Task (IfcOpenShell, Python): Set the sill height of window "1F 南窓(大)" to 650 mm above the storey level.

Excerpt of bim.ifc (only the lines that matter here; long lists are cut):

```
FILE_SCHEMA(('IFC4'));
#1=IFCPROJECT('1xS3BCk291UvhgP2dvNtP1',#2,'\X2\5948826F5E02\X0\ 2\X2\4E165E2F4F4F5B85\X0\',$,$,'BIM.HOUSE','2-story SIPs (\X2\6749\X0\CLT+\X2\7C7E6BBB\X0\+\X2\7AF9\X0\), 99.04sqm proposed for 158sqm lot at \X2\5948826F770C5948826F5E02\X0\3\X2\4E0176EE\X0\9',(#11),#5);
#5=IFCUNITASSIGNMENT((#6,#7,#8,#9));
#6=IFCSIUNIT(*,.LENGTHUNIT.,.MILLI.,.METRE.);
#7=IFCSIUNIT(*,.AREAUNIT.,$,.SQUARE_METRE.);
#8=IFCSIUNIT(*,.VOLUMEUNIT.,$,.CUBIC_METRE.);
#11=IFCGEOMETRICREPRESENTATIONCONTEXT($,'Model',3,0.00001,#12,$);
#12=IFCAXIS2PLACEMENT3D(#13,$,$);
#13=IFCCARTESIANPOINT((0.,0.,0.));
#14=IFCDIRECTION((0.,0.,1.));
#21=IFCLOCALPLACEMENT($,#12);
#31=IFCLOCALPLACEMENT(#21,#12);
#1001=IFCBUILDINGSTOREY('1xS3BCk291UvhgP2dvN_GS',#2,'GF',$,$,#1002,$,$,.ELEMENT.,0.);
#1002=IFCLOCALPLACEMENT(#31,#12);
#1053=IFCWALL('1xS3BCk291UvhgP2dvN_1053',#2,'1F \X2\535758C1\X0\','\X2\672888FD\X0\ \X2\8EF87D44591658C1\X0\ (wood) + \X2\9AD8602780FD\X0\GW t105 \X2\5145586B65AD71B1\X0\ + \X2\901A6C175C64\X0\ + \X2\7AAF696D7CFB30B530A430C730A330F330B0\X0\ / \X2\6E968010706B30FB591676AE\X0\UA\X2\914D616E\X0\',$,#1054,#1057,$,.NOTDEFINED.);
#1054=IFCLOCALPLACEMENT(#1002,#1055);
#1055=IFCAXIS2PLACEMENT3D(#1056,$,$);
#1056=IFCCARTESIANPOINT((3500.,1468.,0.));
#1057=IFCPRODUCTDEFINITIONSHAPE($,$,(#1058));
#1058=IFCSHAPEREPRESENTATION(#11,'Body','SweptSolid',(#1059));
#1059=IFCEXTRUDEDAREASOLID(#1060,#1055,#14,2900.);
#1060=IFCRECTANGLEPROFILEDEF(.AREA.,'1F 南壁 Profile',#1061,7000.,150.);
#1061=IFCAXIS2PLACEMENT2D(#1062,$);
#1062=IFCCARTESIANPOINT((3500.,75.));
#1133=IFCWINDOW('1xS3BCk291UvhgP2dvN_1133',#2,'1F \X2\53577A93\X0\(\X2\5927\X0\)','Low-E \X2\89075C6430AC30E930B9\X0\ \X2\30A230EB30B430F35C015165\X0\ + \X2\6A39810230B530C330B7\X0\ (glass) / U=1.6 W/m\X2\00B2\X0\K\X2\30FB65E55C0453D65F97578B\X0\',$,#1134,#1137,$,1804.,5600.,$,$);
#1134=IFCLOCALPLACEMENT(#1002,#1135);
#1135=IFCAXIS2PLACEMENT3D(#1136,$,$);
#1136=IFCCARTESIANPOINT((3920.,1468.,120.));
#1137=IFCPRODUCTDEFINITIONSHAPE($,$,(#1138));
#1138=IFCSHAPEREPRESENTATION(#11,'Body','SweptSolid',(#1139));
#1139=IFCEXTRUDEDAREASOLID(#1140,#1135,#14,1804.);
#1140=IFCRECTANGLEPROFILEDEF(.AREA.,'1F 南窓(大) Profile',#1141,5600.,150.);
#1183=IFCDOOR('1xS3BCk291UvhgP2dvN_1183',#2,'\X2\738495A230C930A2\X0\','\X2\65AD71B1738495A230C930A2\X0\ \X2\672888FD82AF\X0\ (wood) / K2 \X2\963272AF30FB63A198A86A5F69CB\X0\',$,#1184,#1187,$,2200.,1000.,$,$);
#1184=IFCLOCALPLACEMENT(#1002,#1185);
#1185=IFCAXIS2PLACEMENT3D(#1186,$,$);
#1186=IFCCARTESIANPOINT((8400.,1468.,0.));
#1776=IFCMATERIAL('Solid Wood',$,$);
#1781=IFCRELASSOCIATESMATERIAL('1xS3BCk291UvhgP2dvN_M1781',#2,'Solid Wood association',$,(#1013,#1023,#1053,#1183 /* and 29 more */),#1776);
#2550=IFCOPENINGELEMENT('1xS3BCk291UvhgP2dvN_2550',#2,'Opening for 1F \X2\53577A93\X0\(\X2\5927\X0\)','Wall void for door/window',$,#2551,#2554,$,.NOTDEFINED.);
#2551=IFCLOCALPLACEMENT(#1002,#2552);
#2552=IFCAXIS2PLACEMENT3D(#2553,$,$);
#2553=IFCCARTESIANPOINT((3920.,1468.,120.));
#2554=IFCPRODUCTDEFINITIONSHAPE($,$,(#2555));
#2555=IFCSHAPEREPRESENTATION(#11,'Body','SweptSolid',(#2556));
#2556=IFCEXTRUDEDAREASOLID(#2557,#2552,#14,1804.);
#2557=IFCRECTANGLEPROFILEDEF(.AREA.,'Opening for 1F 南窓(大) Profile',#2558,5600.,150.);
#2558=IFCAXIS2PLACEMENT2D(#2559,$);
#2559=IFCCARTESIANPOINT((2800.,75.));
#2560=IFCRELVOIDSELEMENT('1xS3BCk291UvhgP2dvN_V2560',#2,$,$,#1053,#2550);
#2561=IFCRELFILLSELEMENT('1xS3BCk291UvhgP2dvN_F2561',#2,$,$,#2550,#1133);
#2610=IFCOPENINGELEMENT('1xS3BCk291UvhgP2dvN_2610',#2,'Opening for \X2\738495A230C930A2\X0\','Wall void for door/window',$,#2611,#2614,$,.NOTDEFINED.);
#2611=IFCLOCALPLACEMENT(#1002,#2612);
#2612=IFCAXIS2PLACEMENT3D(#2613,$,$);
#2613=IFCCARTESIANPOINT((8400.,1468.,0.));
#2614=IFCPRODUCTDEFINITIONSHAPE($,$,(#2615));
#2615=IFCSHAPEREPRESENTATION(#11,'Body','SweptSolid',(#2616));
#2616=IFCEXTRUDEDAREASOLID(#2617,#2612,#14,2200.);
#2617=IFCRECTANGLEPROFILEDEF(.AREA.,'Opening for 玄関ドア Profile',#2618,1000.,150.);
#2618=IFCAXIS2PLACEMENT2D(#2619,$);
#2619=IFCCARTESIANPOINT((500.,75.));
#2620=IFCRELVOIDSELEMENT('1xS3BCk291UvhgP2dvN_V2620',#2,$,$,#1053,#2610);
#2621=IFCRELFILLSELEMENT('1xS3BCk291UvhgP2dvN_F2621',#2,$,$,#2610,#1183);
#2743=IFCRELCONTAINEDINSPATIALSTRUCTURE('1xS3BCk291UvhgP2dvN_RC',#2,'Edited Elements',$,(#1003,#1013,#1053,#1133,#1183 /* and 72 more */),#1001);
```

```python
import numpy as np
import ifcopenshell
import ifcopenshell.api.geometry
import ifcopenshell.geom
import ifcopenshell.util.element
import ifcopenshell.util.placement
import ifcopenshell.util.shape
import ifcopenshell.util.unit

model = ifcopenshell.open("bim.ifc")
unit_scale = ifcopenshell.util.unit.calculate_unit_scale(model)

window = model.by_guid("1xS3BCk291UvhgP2dvN_1133")
opening = window.FillsVoids[0].RelatingOpeningElement
storey = ifcopenshell.util.element.get_container(window, ifc_class="IfcBuildingStorey")
level = ifcopenshell.util.placement.get_local_placement(storey.ObjectPlacement)[2, 3]

# The opening's origin need not be at the sill, so measure its lowest point.
shape = ifcopenshell.geom.create_shape(ifcopenshell.geom.settings(), opening)
bottom = ifcopenshell.util.shape.get_shape_bottom_elevation(shape, shape.geometry) / unit_scale
dz = level + 0.65 / unit_scale - bottom

shift = np.array([0.0, 0.0, dz])
# The window is not placed relative to its opening, so move both.
for product in (opening, window):
    matrix = ifcopenshell.util.placement.get_local_placement(product.ObjectPlacement)
    matrix[:3, 3] += shift
    ifcopenshell.api.geometry.edit_object_placement(model, product=product, matrix=matrix, is_si=False)

print(f"moved by {dz * unit_scale:+.3f} m")

model.write("bim_updated.ifc")
```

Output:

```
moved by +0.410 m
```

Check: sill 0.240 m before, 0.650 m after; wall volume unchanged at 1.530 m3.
